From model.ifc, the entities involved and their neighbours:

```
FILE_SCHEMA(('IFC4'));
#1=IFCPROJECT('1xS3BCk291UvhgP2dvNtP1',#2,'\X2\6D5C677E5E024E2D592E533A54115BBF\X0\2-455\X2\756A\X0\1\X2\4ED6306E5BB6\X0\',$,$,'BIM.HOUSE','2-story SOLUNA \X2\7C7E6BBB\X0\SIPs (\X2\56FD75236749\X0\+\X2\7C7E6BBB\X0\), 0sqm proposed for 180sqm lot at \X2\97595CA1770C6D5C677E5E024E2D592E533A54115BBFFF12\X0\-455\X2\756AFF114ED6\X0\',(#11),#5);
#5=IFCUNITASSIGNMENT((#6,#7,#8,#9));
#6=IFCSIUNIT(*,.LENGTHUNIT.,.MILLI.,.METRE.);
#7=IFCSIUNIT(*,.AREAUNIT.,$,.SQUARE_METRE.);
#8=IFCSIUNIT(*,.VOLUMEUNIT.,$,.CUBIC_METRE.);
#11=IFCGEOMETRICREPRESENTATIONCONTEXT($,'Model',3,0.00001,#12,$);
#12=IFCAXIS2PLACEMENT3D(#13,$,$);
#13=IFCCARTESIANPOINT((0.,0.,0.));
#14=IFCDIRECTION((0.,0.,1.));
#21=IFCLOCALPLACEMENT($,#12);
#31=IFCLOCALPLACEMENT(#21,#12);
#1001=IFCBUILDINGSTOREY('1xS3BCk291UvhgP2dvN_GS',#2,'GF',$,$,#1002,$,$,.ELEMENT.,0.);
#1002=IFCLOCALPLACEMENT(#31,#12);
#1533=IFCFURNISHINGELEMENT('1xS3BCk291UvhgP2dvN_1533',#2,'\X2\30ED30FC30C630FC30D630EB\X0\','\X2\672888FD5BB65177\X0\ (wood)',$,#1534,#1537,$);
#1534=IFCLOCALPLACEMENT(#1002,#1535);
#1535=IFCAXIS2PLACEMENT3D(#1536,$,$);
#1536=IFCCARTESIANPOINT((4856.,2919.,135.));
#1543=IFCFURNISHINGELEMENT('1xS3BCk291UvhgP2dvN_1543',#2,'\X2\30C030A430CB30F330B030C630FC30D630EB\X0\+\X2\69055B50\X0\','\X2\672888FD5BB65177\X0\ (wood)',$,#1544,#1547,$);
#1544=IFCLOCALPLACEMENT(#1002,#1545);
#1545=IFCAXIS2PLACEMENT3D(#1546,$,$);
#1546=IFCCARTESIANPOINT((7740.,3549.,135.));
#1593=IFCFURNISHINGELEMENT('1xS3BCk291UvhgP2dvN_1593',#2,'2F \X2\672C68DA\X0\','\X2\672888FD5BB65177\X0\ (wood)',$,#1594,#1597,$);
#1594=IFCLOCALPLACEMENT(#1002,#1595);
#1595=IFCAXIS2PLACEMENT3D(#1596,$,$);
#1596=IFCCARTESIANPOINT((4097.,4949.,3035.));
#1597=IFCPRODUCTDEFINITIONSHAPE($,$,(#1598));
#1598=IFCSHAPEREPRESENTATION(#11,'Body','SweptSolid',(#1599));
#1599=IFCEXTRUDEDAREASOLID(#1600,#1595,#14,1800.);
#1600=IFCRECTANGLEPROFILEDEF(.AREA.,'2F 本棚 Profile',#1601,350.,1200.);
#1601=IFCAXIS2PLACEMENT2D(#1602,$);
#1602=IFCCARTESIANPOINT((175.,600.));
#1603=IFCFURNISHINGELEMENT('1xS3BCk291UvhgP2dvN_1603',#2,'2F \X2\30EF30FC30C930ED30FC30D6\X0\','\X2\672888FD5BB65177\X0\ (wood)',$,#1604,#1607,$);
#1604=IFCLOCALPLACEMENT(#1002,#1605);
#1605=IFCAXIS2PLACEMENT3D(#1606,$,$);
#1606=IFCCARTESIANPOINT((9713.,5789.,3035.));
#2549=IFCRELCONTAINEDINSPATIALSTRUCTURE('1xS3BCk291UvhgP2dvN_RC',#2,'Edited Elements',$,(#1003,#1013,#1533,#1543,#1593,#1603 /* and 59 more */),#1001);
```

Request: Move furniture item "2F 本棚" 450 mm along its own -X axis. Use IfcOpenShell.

```python
import ifcopenshell
import ifcopenshell.api.geometry
import ifcopenshell.util.placement
import ifcopenshell.util.unit

model = ifcopenshell.open("model.ifc")
unit_scale = ifcopenshell.util.unit.calculate_unit_scale(model)

item = model.by_guid("1xS3BCk291UvhgP2dvN_1593")
matrix = ifcopenshell.util.placement.get_local_placement(item.ObjectPlacement)
matrix[:3, 3] -= matrix[:3, 0] * 0.45 / unit_scale
ifcopenshell.api.geometry.edit_object_placement(model, product=item, matrix=matrix, is_si=False)

print(ifcopenshell.util.placement.get_local_placement(item.ObjectPlacement).round(3) + 0.0)

model.write("model_updated.ifc")
```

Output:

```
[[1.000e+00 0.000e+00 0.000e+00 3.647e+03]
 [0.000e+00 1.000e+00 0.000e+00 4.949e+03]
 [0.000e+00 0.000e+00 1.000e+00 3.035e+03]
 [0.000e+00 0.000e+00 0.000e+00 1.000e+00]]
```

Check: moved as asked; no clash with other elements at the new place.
